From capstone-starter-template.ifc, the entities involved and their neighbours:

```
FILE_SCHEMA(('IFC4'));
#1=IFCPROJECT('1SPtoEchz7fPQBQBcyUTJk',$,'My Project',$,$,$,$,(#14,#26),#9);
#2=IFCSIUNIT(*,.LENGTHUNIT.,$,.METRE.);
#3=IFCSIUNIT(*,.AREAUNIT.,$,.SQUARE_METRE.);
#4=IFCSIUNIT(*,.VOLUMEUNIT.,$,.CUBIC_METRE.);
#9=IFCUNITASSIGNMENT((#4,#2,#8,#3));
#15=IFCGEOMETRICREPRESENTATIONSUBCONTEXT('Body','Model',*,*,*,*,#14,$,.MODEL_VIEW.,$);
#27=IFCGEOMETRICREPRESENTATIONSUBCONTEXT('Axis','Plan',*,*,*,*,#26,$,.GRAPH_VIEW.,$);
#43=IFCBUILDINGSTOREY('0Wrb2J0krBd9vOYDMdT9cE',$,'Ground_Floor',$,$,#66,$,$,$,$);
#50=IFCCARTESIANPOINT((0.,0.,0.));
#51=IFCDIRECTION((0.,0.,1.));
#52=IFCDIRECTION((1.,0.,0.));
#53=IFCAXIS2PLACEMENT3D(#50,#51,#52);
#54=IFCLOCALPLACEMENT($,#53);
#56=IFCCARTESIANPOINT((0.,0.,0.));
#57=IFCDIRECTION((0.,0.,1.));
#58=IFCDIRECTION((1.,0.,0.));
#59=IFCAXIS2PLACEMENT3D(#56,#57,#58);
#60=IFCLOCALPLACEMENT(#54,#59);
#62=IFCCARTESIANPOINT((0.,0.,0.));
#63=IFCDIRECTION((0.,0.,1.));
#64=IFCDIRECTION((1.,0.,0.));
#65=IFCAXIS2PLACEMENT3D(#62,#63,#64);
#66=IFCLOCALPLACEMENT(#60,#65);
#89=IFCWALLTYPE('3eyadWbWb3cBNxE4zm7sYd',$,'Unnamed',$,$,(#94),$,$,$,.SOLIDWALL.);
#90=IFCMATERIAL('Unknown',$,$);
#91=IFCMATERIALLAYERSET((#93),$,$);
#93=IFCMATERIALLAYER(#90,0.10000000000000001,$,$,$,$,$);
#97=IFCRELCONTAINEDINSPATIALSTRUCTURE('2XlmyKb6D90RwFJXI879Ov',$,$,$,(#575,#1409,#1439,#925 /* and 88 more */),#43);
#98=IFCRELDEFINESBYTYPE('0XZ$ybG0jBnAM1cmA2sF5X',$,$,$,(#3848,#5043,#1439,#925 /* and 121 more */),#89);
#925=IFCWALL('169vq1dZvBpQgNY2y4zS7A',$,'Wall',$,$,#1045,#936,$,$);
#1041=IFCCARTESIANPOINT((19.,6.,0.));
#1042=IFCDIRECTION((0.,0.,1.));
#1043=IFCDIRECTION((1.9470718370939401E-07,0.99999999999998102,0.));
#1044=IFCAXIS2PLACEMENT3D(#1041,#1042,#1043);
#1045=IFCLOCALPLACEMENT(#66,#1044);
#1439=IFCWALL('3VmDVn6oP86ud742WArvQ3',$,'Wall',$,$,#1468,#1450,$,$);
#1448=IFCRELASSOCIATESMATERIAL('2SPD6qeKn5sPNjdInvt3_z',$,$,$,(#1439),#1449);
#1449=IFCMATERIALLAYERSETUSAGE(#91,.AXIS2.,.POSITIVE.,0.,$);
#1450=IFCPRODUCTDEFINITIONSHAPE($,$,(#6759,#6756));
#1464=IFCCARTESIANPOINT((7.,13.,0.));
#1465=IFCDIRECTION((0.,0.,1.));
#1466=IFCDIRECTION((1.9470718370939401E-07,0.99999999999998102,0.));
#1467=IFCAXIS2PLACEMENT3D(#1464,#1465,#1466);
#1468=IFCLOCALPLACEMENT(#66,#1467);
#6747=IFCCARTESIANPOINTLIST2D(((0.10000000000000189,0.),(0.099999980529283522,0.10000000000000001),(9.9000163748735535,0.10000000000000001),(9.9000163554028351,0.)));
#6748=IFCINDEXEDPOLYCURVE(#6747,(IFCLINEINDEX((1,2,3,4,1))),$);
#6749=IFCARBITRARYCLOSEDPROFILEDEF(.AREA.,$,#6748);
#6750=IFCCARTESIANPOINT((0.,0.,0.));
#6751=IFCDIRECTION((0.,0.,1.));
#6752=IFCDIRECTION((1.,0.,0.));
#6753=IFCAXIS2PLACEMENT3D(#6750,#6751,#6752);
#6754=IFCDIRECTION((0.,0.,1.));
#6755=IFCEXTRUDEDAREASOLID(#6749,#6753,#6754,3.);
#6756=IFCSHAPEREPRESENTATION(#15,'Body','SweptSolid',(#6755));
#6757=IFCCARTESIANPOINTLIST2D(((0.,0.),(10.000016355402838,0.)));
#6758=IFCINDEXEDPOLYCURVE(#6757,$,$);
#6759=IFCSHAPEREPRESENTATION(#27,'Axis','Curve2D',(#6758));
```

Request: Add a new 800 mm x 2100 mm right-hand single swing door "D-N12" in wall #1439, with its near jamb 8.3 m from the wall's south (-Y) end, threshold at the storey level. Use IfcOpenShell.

```python
import numpy as np
import ifcopenshell
import ifcopenshell.api.feature
import ifcopenshell.api.geometry
import ifcopenshell.api.root
import ifcopenshell.api.spatial
import ifcopenshell.geom
import ifcopenshell.util.element
import ifcopenshell.util.placement
import ifcopenshell.util.representation
import ifcopenshell.util.shape
import ifcopenshell.util.unit

model = ifcopenshell.open("capstone-starter-template.ifc")
unit_scale = ifcopenshell.util.unit.calculate_unit_scale(model)
settings = ifcopenshell.geom.settings()


def volume(element):
    """Net volume in cubic metres, openings subtracted."""
    shape = ifcopenshell.geom.create_shape(settings, element)
    return ifcopenshell.util.shape.get_volume(shape.geometry)


wall = model.by_guid("3VmDVn6oP86ud742WArvQ3")
storey = ifcopenshell.util.element.get_container(wall, ifc_class="IfcBuildingStorey")
context = ifcopenshell.util.representation.get_context(model, "Model", "Body", "MODEL_VIEW")
before = volume(wall)

width, height, from_end, sill = 0.8, 2.1, 8.3, 0.0  # metres

# The wall runs along its own X axis, and the end named is its -X end.
wall_shape = ifcopenshell.geom.create_shape(settings, wall)
x, y, z = ifcopenshell.util.shape.get_vertices(wall_shape.geometry).T
start = x.min() + from_end
face, thickness = float(y.min()), float(y.max() - y.min())
wall_matrix = ifcopenshell.util.placement.get_local_placement(wall.ObjectPlacement)
level = ifcopenshell.util.placement.get_local_placement(storey.ObjectPlacement)[2, 3]


def in_wall(x, y):
    """Placement at x, y metres in the wall's axes, at sill height."""
    matrix = wall_matrix.copy()
    matrix[:, 3] = wall_matrix @ np.array([x / unit_scale, y / unit_scale, 0.0, 1.0])
    matrix[2, 3] = level + sill / unit_scale
    return matrix


# Opening: a box that overshoots both wall faces by 50 mm.
opening = ifcopenshell.api.root.create_entity(model, ifc_class="IfcOpeningElement", predefined_type="OPENING")
box = ifcopenshell.api.geometry.add_wall_representation(
    model, context=context, length=width, height=height, thickness=thickness + 0.1
)
ifcopenshell.api.geometry.assign_representation(model, product=opening, representation=box)
ifcopenshell.api.geometry.edit_object_placement(model, product=opening, matrix=in_wall(start, face - 0.05), is_si=False)
ifcopenshell.api.feature.add_feature(model, feature=opening, element=wall)

door = ifcopenshell.api.root.create_entity(model, ifc_class="IfcDoor", name="D-N12", predefined_type="DOOR")
door.OverallWidth, door.OverallHeight = width / unit_scale, height / unit_scale
door.OperationType = "SINGLE_SWING_RIGHT"
body = ifcopenshell.api.geometry.add_door_representation(
    model,
    context=context,
    overall_width=door.OverallWidth,
    overall_height=door.OverallHeight,
    operation_type="SINGLE_SWING_RIGHT",
    lining_properties={"LiningDepth": thickness / unit_scale, "ThresholdDepth": thickness / unit_scale},
)
ifcopenshell.api.geometry.assign_representation(model, product=door, representation=body)
ifcopenshell.api.spatial.assign_container(model, products=[door], relating_structure=storey)
ifcopenshell.api.feature.add_filling(model, opening=opening, element=door)

# The lining spans the wall, so the door starts at the wall face.
ifcopenshell.api.geometry.edit_object_placement(model, product=door, matrix=in_wall(start, face), is_si=False)

after = volume(wall)

print(f"wall volume {before:.3f} -> {after:.3f} m3")

model.write("capstone-starter-template_edited.ifc")
```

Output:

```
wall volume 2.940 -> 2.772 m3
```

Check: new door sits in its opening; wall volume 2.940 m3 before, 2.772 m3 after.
